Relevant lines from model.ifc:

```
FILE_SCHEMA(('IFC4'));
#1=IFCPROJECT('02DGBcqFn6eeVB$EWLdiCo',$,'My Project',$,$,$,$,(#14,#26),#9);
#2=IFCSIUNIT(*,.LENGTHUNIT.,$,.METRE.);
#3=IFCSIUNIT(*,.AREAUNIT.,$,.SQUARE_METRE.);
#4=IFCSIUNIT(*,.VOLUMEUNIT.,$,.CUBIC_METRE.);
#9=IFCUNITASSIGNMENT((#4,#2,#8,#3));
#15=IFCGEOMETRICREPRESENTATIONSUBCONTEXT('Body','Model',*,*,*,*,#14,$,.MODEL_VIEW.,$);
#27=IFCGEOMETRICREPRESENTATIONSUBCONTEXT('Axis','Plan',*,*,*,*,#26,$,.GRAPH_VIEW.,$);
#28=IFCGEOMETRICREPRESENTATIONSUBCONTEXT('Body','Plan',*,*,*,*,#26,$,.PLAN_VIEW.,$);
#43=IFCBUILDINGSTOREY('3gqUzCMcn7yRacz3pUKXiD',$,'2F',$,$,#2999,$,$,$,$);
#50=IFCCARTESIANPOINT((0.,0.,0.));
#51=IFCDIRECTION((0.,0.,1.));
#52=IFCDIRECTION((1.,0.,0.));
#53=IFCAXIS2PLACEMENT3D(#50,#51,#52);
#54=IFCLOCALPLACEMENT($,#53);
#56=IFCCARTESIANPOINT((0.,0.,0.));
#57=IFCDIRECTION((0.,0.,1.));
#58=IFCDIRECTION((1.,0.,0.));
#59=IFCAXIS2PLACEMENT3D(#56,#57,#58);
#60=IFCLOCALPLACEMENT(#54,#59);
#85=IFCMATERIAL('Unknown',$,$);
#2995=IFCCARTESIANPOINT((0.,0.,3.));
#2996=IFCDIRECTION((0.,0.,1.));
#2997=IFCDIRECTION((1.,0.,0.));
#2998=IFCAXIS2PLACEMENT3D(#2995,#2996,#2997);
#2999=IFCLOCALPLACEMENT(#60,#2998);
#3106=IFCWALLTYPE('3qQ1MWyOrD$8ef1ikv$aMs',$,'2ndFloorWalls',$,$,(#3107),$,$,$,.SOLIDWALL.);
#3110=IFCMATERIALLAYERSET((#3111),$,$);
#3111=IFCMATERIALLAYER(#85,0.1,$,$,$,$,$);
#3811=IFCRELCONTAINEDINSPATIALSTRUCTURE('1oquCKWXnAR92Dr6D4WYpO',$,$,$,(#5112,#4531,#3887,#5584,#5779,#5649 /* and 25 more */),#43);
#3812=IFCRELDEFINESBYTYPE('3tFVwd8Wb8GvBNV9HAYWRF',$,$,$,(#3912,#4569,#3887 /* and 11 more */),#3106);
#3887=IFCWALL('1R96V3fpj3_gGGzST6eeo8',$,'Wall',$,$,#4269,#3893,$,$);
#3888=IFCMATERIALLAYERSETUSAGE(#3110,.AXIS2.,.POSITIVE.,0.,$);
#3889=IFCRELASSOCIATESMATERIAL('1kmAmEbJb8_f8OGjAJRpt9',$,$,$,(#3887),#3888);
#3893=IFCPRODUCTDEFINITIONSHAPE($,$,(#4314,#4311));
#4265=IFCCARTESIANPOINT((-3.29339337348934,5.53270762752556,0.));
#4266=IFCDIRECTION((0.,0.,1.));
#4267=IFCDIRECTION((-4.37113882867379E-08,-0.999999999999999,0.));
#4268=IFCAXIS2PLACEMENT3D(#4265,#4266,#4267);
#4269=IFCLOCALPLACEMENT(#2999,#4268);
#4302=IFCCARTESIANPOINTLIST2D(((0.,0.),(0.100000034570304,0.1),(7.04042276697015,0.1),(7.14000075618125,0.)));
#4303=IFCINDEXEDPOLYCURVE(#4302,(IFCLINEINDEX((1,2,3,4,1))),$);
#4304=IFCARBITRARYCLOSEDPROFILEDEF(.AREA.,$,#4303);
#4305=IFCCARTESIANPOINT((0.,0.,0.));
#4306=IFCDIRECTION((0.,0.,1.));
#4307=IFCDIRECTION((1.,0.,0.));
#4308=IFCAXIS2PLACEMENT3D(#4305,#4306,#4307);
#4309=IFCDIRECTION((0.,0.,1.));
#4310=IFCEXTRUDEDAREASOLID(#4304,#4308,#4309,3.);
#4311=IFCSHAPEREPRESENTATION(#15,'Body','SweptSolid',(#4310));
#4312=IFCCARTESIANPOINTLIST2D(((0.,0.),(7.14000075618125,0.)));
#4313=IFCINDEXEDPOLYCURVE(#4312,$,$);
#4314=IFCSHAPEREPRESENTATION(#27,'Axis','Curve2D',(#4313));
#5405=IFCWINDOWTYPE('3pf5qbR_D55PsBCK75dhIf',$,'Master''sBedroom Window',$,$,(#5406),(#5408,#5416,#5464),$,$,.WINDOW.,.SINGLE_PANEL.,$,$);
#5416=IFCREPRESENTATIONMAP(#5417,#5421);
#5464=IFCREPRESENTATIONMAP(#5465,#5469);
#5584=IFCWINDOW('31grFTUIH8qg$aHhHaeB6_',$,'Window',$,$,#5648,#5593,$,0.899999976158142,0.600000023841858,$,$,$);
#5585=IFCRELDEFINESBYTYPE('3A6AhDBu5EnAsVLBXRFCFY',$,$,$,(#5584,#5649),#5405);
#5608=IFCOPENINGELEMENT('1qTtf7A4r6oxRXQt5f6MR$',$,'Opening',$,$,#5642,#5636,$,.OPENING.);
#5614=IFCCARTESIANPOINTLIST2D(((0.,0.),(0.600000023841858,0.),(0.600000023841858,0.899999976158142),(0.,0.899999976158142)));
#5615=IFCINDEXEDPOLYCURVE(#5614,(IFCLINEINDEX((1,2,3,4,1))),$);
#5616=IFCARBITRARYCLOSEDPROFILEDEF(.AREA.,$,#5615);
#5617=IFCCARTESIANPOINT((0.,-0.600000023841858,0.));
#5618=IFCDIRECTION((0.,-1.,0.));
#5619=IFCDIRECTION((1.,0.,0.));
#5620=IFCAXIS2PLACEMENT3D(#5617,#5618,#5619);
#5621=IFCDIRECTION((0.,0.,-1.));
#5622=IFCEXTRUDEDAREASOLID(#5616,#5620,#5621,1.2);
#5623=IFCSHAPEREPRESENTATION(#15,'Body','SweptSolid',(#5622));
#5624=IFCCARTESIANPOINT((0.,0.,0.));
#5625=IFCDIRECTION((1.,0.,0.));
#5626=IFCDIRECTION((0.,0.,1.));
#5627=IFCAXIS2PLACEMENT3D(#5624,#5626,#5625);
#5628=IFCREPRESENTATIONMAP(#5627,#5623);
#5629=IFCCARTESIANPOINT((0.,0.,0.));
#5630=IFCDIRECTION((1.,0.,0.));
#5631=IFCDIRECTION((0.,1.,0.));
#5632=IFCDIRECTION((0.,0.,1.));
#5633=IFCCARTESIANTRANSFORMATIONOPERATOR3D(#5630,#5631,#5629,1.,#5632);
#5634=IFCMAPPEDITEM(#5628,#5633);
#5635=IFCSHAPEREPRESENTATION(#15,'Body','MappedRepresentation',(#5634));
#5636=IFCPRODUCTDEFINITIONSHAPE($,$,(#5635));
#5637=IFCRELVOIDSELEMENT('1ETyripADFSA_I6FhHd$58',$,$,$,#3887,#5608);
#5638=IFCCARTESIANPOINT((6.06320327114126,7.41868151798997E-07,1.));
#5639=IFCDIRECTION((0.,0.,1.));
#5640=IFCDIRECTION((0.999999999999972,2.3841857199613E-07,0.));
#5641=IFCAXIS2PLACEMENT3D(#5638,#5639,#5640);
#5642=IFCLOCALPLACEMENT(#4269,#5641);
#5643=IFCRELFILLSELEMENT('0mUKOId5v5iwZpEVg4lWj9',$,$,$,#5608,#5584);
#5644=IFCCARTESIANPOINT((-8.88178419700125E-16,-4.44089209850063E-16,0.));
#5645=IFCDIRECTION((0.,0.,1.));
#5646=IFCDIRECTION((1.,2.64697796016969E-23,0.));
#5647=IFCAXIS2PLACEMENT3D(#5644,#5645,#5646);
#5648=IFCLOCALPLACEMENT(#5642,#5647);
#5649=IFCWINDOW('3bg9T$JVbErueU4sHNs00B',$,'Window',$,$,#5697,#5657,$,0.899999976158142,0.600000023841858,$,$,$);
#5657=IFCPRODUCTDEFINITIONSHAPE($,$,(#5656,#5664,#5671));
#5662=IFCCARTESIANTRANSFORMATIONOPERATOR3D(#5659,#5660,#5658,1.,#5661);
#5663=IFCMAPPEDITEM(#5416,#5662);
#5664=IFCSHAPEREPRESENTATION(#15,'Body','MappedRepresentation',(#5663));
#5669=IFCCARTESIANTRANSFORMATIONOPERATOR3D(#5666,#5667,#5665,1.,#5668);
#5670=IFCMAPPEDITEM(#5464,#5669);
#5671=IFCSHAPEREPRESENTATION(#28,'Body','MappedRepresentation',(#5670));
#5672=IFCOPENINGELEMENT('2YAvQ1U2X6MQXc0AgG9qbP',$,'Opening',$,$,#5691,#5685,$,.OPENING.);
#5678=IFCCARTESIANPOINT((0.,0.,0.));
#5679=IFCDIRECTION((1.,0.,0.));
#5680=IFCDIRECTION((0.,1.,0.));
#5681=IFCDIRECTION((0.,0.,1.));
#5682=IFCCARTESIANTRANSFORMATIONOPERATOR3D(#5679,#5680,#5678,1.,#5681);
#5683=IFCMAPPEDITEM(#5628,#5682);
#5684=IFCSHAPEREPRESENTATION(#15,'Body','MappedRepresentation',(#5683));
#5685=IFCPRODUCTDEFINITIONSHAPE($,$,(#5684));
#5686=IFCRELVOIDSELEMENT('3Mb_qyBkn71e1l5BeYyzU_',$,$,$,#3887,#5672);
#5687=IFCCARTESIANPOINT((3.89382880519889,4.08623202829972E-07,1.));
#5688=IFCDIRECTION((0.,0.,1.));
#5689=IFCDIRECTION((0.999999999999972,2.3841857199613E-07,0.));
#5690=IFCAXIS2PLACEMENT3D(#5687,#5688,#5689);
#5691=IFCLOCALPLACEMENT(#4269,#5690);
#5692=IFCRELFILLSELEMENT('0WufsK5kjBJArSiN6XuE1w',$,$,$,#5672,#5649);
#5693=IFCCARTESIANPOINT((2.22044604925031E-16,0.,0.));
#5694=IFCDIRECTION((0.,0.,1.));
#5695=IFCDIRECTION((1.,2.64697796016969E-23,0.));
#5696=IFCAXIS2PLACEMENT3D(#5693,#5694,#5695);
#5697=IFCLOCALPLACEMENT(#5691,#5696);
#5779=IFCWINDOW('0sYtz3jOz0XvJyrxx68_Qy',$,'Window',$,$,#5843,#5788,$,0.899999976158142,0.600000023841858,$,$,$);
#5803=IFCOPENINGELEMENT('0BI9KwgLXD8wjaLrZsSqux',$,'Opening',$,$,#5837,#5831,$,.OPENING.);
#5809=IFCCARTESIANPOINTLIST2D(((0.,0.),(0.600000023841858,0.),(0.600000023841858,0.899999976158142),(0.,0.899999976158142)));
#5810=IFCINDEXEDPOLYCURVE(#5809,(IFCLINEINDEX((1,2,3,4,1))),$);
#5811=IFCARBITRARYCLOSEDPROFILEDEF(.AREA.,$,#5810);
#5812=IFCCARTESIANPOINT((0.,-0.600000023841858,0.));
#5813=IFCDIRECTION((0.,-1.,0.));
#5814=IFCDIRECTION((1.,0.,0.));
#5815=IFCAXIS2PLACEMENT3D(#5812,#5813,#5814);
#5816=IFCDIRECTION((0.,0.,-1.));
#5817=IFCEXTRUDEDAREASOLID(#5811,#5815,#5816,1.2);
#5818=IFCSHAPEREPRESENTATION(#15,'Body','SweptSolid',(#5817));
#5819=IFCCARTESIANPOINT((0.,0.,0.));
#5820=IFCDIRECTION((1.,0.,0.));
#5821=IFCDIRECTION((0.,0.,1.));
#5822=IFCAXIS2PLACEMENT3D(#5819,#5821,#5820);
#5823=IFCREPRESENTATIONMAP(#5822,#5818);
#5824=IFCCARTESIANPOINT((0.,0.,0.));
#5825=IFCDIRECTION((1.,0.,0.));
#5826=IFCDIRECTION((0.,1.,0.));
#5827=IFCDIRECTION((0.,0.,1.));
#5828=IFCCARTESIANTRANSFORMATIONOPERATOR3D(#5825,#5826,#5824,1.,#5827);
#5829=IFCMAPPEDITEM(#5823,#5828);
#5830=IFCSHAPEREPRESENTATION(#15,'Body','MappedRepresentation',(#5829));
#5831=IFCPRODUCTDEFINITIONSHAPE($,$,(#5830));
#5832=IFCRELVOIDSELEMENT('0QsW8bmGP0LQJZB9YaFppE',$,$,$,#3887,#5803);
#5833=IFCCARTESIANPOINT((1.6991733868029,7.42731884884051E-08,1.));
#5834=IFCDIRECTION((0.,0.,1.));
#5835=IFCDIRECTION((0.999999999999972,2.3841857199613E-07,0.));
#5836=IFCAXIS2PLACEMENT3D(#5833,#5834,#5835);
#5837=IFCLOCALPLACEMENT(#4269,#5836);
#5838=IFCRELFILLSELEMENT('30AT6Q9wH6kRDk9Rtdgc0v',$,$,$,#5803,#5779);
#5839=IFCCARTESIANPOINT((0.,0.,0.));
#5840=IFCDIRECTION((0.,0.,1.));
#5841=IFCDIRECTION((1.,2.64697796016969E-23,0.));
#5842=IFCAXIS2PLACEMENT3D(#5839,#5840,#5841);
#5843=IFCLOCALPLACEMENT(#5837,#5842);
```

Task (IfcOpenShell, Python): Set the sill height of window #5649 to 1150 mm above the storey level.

```python
import numpy as np
import ifcopenshell
import ifcopenshell.api.geometry
import ifcopenshell.geom
import ifcopenshell.util.element
import ifcopenshell.util.placement
import ifcopenshell.util.shape
import ifcopenshell.util.unit

model = ifcopenshell.open("model.ifc")
unit_scale = ifcopenshell.util.unit.calculate_unit_scale(model)

window = model.by_guid("3bg9T$JVbErueU4sHNs00B")
opening = window.FillsVoids[0].RelatingOpeningElement
storey = ifcopenshell.util.element.get_container(window, ifc_class="IfcBuildingStorey")
level = ifcopenshell.util.placement.get_local_placement(storey.ObjectPlacement)[2, 3]

# The opening's origin need not be at the sill, so measure its lowest point.
shape = ifcopenshell.geom.create_shape(ifcopenshell.geom.settings(), opening)
bottom = ifcopenshell.util.shape.get_shape_bottom_elevation(shape, shape.geometry) / unit_scale
dz = level + 1.15 / unit_scale - bottom

shift = np.array([0.0, 0.0, dz])
# The window is placed relative to its opening, so it follows when the opening moves.
matrix = ifcopenshell.util.placement.get_local_placement(opening.ObjectPlacement)
matrix[:3, 3] += shift
ifcopenshell.api.geometry.edit_object_placement(
    model, product=opening, matrix=matrix, is_si=False, should_transform_children=True
)

print(f"moved by {dz * unit_scale:+.3f} m")

model.write("model_edited.ifc")
```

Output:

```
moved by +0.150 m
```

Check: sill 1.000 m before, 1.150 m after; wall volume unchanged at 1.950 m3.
